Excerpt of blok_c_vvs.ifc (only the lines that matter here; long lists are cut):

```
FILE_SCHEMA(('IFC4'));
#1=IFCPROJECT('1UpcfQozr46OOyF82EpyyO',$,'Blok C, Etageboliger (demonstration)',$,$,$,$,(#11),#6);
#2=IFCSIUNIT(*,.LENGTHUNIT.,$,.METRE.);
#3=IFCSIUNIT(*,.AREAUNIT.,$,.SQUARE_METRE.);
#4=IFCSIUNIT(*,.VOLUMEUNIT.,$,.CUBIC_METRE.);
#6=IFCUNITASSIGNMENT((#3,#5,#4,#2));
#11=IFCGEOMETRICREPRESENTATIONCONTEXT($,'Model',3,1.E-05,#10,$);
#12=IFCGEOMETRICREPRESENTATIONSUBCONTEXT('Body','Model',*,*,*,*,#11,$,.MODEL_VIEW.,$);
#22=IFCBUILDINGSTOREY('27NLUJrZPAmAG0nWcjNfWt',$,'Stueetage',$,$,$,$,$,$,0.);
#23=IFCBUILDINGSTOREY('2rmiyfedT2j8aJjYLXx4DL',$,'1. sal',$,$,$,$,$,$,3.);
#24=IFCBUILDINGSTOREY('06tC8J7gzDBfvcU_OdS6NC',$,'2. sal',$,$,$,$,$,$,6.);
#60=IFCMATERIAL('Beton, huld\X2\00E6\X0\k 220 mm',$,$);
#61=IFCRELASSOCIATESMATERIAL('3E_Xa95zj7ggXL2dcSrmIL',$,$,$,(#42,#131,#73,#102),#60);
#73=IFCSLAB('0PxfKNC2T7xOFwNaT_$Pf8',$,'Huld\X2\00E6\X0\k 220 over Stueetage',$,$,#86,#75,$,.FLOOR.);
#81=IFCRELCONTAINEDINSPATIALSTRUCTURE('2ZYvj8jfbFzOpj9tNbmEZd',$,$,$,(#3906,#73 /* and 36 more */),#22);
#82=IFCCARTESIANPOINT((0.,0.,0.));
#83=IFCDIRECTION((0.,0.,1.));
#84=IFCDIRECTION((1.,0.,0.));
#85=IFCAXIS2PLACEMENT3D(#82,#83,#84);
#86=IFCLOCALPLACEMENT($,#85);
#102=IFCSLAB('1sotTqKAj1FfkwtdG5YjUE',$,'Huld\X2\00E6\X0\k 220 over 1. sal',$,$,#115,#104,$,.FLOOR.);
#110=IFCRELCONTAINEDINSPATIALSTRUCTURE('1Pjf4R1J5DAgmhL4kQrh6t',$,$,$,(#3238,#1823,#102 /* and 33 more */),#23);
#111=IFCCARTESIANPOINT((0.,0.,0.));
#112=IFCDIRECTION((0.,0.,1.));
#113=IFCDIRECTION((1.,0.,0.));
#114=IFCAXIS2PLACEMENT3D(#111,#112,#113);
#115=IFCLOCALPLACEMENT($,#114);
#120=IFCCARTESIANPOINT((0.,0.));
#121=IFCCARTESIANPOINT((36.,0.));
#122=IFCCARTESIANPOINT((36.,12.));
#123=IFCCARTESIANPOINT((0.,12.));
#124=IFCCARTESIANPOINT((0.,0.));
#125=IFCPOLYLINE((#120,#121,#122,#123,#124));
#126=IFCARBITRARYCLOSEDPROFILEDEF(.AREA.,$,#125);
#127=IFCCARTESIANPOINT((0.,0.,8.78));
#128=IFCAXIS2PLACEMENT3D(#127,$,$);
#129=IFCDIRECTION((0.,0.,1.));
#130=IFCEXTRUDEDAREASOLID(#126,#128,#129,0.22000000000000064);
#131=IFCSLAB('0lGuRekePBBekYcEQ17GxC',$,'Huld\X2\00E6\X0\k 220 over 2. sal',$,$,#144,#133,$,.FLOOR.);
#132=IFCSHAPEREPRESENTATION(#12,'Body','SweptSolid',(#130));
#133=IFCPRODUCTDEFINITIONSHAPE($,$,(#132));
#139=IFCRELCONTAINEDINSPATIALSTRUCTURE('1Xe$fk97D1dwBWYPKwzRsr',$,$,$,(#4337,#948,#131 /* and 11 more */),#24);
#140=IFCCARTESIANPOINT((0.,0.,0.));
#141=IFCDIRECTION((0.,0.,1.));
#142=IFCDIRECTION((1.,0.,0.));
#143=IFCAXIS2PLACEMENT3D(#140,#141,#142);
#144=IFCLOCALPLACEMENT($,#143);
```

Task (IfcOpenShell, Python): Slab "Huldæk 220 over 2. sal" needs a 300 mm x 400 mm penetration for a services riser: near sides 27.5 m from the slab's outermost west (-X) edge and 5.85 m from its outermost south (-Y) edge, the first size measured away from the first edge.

```python
import numpy as np
import ifcopenshell
import ifcopenshell.api.feature
import ifcopenshell.api.geometry
import ifcopenshell.api.root
import ifcopenshell.geom
import ifcopenshell.util.placement
import ifcopenshell.util.representation
import ifcopenshell.util.shape
import ifcopenshell.util.unit

model = ifcopenshell.open("blok_c_vvs.ifc")
unit_scale = ifcopenshell.util.unit.calculate_unit_scale(model)
settings = ifcopenshell.geom.settings()


def volume(element):
    """Net volume in cubic metres, openings subtracted."""
    shape = ifcopenshell.geom.create_shape(settings, element)
    return ifcopenshell.util.shape.get_volume(shape.geometry)


slab = model.by_guid("0lGuRekePBBekYcEQ17GxC")
before = volume(slab)

# Extent in the slab's own axes, in metres. The edges named are its -X and -Y sides.
slab_shape = ifcopenshell.geom.create_shape(settings, slab)
vertices = ifcopenshell.util.shape.get_vertices(slab_shape.geometry)
x_min, y_min, bottom = vertices.min(axis=0)
top = vertices[:, 2].max()

opening = ifcopenshell.api.root.create_entity(model, ifc_class="IfcOpeningElement", name="Services riser opening", predefined_type="OPENING")
context = ifcopenshell.util.representation.get_context(model, "Model", "Body", "MODEL_VIEW")
width, depth = 0.3, 0.4
outline = [(0.0, 0.0), (width, 0.0), (width, depth), (0.0, depth), (0.0, 0.0)]
# Overshoot both faces by 50 mm so the cut is clean.
shape = ifcopenshell.api.geometry.add_slab_representation(
    model, context=context, depth=top - bottom + 0.1, polyline=outline
)
ifcopenshell.api.geometry.assign_representation(model, product=opening, representation=shape)

matrix = ifcopenshell.util.placement.get_local_placement(slab.ObjectPlacement)
matrix[:, 3] = matrix @ np.append(np.array([x_min + 27.5, y_min + 5.85, bottom - 0.05]) / unit_scale, 1.0)
ifcopenshell.api.geometry.edit_object_placement(model, product=opening, matrix=matrix, is_si=False)
ifcopenshell.api.feature.add_feature(model, feature=opening, element=slab)

after = volume(slab)

print(f"slab volume {before:.3f} -> {after:.3f} m3")

model.write("blok_c_vvs_updated.ifc")
```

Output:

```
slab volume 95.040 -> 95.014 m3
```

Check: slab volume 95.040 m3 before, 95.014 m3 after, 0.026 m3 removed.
